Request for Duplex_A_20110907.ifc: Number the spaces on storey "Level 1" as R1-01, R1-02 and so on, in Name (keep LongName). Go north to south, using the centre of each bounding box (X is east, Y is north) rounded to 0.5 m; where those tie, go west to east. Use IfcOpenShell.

First a look at what the model holds.

```python
import ifcopenshell
import ifcopenshell.util.element
import ifcopenshell.util.placement

model = ifcopenshell.open("Duplex_A_20110907.ifc")
print(model.schema)
storey = next(s for s in model.by_type("IfcBuildingStorey") if s.Name == "Level 1")
spaces = [e for e in ifcopenshell.util.element.get_decomposition(storey) if e.is_a("IfcSpace")]
for e in sorted(spaces, key=lambda e: e.id()):
    origin = ifcopenshell.util.placement.get_local_placement(e.ObjectPlacement)[:3, 3]
    print(e.id(), e.Name, e.LongName, origin.round(2) + 0.0, sep=" | ")
```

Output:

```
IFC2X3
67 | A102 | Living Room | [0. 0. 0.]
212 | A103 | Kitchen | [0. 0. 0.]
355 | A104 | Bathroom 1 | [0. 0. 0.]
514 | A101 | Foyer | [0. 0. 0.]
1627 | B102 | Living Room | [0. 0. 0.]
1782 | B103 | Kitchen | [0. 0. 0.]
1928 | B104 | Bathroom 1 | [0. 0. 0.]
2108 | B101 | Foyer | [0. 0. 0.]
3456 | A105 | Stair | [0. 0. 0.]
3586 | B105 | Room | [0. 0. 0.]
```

```python
import ifcopenshell
import ifcopenshell.geom
import ifcopenshell.util.element
import ifcopenshell.util.shape

model = ifcopenshell.open("Duplex_A_20110907.ifc")
settings = ifcopenshell.geom.settings()
settings.set("use-world-coords", True)


def centre(element):
    shape = ifcopenshell.geom.create_shape(settings, element)
    return ifcopenshell.util.shape.get_bbox_centroid(shape.geometry)


storey = next(s for s in model.by_type("IfcBuildingStorey") if s.Name == "Level 1")
spaces = [e for e in ifcopenshell.util.element.get_decomposition(storey) if e.is_a("IfcSpace")]

# Insertion points can sit at a corner or the storey origin, so sort by the geometry (in metres).
centres = {e: centre(e) for e in spaces}
spaces.sort(key=lambda e: (-round(centres[e][1] / 0.5), centres[e][0]))

for i, e in enumerate(spaces, start=1):
    number = f"R1-{i:02d}"
    e.Name = number
    print(e.id(), number)

model.write("Duplex_A_20110907_edited.ifc")
```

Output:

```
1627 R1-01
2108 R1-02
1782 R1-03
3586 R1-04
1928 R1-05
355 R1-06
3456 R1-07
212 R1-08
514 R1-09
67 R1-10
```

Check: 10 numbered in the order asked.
